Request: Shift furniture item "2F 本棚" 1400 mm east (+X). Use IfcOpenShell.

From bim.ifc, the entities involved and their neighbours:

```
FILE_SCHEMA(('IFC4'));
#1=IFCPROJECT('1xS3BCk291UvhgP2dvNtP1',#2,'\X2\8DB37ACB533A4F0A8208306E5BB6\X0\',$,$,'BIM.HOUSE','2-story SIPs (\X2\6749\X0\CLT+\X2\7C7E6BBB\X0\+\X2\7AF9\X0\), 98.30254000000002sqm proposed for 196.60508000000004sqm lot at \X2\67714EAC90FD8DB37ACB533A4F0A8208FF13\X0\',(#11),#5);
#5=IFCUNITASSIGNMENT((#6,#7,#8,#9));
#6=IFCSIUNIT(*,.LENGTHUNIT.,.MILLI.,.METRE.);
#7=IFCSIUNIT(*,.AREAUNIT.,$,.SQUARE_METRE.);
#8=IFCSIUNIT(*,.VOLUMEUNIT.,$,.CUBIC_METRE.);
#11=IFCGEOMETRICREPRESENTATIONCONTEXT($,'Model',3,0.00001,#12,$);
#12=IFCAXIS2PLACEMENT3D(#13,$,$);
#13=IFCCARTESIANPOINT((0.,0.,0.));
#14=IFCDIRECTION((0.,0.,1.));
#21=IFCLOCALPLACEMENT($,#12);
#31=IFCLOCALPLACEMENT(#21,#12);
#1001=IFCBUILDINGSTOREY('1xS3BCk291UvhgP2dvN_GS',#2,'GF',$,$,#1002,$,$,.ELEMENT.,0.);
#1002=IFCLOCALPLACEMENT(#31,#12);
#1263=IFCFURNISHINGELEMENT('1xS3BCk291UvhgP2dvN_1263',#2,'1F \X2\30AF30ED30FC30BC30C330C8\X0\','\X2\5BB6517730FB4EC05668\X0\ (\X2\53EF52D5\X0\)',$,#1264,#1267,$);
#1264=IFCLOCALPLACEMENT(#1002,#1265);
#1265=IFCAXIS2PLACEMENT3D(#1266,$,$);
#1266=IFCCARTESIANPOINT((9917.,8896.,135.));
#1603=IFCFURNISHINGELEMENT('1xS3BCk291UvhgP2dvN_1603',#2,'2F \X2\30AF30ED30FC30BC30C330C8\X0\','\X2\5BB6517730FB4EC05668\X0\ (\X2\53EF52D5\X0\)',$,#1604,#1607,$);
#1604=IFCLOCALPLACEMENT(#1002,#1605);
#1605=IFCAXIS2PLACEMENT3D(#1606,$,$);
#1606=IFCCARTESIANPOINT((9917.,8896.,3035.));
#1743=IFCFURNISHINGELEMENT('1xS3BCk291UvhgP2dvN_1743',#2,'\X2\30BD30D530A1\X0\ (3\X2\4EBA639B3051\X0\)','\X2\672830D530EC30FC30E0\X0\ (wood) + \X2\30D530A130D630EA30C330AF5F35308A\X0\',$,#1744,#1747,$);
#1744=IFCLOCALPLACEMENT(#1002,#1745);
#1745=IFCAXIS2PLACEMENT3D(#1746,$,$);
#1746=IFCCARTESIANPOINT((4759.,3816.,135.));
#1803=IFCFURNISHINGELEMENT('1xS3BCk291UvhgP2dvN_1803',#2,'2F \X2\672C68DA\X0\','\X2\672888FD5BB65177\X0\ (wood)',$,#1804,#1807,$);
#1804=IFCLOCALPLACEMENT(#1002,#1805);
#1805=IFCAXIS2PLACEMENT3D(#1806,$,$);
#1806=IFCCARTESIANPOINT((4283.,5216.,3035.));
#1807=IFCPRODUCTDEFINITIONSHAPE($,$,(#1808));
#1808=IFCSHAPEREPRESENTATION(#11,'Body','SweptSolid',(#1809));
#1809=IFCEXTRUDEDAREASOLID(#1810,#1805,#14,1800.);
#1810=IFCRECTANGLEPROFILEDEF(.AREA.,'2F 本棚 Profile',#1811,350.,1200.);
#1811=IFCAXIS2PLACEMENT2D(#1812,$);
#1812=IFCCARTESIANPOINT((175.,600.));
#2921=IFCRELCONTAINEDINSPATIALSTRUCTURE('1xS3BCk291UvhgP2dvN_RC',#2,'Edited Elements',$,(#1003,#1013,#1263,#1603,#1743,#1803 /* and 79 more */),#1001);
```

```python
import ifcopenshell
import ifcopenshell.api.geometry
import ifcopenshell.util.placement

model = ifcopenshell.open("bim.ifc")

item = model.by_id(1803)
matrix = ifcopenshell.util.placement.get_local_placement(item.ObjectPlacement)
matrix[0, 3] += 1400.0
ifcopenshell.api.geometry.edit_object_placement(model, product=item, matrix=matrix, is_si=False)

print(ifcopenshell.util.placement.get_local_placement(item.ObjectPlacement).round(3) + 0.0)

model.write("bim_updated.ifc")
```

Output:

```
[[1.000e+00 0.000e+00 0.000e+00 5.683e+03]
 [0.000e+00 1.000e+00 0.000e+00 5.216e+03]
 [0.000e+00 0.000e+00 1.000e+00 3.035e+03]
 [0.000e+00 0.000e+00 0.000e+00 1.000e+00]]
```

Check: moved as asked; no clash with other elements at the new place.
